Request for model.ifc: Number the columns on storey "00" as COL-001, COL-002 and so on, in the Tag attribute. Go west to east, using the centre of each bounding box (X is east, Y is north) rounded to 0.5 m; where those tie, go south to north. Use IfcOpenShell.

First a look at what the model holds.

```python
import ifcopenshell
import ifcopenshell.util.element
import ifcopenshell.util.placement

model = ifcopenshell.open("model.ifc")
print(model.schema)
storey = next(s for s in model.by_type("IfcBuildingStorey") if s.Name == "00")
columns = [e for e in ifcopenshell.util.element.get_decomposition(storey) if e.is_a("IfcColumn")]
for e in sorted(columns, key=lambda e: e.id()):
    origin = ifcopenshell.util.placement.get_local_placement(e.ObjectPlacement)[:3, 3]
    print(e.id(), e.Tag, e.Name, origin.round(2) + 0.0, sep=" | ")
```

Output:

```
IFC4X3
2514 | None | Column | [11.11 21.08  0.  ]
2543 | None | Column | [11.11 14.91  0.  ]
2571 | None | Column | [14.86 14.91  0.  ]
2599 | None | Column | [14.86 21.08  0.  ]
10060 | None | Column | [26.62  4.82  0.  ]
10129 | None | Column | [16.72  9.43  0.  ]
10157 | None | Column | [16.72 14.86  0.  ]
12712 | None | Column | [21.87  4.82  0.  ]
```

```python
import ifcopenshell
import ifcopenshell.geom
import ifcopenshell.util.element
import ifcopenshell.util.shape

model = ifcopenshell.open("model.ifc")
settings = ifcopenshell.geom.settings()
settings.set("use-world-coords", True)


def centre(element):
    shape = ifcopenshell.geom.create_shape(settings, element)
    return ifcopenshell.util.shape.get_bbox_centroid(shape.geometry)


storey = next(s for s in model.by_type("IfcBuildingStorey") if s.Name == "00")
columns = [e for e in ifcopenshell.util.element.get_decomposition(storey) if e.is_a("IfcColumn")]

# Insertion points can sit at a corner or the storey origin, so sort by the geometry (in metres).
centres = {e: centre(e) for e in columns}
columns.sort(key=lambda e: (round(centres[e][0] / 0.5), centres[e][1]))

for i, e in enumerate(columns, start=1):
    number = f"COL-0{i:02d}"
    e.Tag = number
    print(e.id(), number)

model.write("model_updated.ifc")
```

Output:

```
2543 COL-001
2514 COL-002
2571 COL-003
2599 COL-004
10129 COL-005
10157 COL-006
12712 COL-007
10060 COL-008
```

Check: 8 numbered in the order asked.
